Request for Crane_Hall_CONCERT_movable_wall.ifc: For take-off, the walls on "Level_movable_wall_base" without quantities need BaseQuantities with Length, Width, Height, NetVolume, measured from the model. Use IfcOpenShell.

First a look at what the model holds.

```python
import ifcopenshell
import ifcopenshell.util.element
import ifcopenshell.util.unit

model = ifcopenshell.open("Crane_Hall_CONCERT_movable_wall.ifc")
print(model.schema)
for unit_type in ("LENGTHUNIT", "AREAUNIT", "VOLUMEUNIT"):
    print(unit_type, ifcopenshell.util.unit.calculate_unit_scale(model, unit_type))
storey = next(s for s in model.by_type("IfcBuildingStorey") if s.Name == "Level_movable_wall_base")
walls = [e for e in ifcopenshell.util.element.get_decomposition(storey) if e.is_a("IfcWall")]
for e in sorted(walls, key=lambda e: e.id()):
    print(e.id(), e.is_a(), e.Name, list(ifcopenshell.util.element.get_psets(e, qtos_only=True)), sep=" | ")
```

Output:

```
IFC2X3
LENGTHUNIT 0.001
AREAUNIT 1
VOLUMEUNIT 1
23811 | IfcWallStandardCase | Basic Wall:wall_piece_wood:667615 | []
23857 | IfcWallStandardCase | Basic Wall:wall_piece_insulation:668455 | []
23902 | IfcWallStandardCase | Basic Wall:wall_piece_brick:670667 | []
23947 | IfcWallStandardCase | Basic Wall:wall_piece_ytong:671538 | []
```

```python
import ifcopenshell
import ifcopenshell.api.pset
import ifcopenshell.geom
import ifcopenshell.util.element
import ifcopenshell.util.shape
import ifcopenshell.util.unit

model = ifcopenshell.open("Crane_Hall_CONCERT_movable_wall.ifc")
unit_scale = ifcopenshell.util.unit.calculate_unit_scale(model)
volume_scale = ifcopenshell.util.unit.calculate_unit_scale(model, "VOLUMEUNIT")
settings = ifcopenshell.geom.settings()

storey = next(s for s in model.by_type("IfcBuildingStorey") if s.Name == "Level_movable_wall_base")
walls = [e for e in ifcopenshell.util.element.get_decomposition(storey) if e.is_a("IfcWall")]

for e in sorted(walls, key=lambda e: e.id()):
    if ifcopenshell.util.element.get_psets(e, qtos_only=True, should_inherit=False):
        continue
    # Geometry comes back in metres, in the element's own axes.
    shape = ifcopenshell.geom.create_shape(settings, e)
    values = {
        "Length": ifcopenshell.util.shape.get_x(shape.geometry) / unit_scale,
        "Width": ifcopenshell.util.shape.get_y(shape.geometry) / unit_scale,
        "Height": ifcopenshell.util.shape.get_z(shape.geometry) / unit_scale,
        "NetVolume": ifcopenshell.util.shape.get_volume(shape.geometry) / volume_scale,
    }
    qto = ifcopenshell.api.pset.add_qto(model, product=e, name="BaseQuantities")
    ifcopenshell.api.pset.edit_qto(model, qto=qto, properties=values)
    print(e.id(), {k: round(v, 3) for k, v in values.items()})

model.write("Crane_Hall_CONCERT_movable_wall-out.ifc")
```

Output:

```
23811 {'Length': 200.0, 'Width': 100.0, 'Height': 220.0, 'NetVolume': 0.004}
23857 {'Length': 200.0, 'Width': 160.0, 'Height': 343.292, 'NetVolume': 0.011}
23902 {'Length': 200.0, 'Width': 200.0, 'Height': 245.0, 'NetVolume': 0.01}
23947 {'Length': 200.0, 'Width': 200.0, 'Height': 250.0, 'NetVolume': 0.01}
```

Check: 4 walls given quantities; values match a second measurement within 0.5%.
